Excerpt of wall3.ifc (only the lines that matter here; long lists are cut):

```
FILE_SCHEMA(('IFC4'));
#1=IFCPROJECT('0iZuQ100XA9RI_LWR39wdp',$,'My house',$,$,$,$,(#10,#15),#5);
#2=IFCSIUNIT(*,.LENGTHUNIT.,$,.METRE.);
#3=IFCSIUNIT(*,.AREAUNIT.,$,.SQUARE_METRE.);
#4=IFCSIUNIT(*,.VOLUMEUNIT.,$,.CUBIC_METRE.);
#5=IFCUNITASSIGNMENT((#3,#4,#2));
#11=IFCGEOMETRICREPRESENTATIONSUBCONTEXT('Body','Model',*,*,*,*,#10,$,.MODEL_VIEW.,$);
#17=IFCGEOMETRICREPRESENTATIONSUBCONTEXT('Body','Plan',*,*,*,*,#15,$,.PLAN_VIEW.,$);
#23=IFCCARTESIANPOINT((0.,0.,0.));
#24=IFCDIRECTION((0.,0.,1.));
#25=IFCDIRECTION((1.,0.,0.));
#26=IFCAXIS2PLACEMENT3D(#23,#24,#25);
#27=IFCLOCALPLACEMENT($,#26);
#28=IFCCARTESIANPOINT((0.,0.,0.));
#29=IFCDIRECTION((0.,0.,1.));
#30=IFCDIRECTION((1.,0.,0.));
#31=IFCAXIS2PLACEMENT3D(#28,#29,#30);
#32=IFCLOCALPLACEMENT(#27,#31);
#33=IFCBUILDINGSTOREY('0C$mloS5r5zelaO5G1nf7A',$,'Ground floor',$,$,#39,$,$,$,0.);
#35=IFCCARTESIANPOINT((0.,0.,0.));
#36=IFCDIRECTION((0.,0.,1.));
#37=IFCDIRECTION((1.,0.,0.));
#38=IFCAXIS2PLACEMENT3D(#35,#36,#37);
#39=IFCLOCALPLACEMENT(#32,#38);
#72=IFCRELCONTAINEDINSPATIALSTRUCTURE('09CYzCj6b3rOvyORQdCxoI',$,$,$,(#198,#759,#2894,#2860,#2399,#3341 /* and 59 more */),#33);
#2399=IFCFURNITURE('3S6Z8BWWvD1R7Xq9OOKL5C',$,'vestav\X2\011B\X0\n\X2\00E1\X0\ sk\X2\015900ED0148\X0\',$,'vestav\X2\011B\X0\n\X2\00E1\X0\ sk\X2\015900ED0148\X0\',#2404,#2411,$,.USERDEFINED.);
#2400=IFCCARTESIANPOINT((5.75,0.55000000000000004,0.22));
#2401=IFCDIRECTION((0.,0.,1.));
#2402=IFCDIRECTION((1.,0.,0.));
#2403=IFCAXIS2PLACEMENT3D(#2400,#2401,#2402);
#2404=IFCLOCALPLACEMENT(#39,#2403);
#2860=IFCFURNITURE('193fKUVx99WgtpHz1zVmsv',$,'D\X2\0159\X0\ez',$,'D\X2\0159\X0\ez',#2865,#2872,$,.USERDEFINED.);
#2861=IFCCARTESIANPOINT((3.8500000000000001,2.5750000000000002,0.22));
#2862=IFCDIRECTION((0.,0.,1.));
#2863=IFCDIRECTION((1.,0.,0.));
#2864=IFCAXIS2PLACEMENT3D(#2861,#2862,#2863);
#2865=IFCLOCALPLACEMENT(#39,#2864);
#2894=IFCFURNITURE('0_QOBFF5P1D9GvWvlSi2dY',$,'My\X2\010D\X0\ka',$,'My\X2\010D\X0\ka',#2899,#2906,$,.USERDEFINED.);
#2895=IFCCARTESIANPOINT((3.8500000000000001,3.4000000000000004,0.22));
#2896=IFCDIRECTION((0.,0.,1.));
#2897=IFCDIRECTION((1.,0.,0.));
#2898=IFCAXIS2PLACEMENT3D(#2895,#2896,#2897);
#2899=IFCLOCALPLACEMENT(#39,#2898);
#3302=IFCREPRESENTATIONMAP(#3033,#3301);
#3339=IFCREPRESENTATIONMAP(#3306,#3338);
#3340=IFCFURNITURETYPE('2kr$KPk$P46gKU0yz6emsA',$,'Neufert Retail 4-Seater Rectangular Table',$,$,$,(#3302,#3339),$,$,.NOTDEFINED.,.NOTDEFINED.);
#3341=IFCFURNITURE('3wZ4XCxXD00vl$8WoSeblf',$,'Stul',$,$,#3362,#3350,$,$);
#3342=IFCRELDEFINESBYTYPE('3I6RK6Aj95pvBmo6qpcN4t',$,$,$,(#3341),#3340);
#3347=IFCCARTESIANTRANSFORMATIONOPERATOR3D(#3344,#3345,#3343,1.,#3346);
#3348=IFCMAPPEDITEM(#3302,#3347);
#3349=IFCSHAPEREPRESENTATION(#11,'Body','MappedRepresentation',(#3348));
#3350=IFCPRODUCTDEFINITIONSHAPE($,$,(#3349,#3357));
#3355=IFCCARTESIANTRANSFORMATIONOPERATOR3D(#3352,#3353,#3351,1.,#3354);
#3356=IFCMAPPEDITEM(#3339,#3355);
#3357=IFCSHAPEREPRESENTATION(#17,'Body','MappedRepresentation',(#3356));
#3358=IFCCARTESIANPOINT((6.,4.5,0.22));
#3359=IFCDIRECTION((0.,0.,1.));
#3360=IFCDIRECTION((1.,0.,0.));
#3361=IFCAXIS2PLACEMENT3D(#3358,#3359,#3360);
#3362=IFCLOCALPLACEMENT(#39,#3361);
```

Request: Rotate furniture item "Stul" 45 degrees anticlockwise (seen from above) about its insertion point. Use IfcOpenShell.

```python
import ifcopenshell
import ifcopenshell.api.geometry
import ifcopenshell.util.placement

model = ifcopenshell.open("wall3.ifc")

item = model.by_guid("3wZ4XCxXD00vl$8WoSeblf")
matrix = ifcopenshell.util.placement.get_local_placement(item.ObjectPlacement)
matrix = matrix @ ifcopenshell.util.placement.rotation(45, "Z")
ifcopenshell.api.geometry.edit_object_placement(model, product=item, matrix=matrix, is_si=False)

print(ifcopenshell.util.placement.get_local_placement(item.ObjectPlacement).round(3) + 0.0)

model.write("wall3_rev.ifc")
```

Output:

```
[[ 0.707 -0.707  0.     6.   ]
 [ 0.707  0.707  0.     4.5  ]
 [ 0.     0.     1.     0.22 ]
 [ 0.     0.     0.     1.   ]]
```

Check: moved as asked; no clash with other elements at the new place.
